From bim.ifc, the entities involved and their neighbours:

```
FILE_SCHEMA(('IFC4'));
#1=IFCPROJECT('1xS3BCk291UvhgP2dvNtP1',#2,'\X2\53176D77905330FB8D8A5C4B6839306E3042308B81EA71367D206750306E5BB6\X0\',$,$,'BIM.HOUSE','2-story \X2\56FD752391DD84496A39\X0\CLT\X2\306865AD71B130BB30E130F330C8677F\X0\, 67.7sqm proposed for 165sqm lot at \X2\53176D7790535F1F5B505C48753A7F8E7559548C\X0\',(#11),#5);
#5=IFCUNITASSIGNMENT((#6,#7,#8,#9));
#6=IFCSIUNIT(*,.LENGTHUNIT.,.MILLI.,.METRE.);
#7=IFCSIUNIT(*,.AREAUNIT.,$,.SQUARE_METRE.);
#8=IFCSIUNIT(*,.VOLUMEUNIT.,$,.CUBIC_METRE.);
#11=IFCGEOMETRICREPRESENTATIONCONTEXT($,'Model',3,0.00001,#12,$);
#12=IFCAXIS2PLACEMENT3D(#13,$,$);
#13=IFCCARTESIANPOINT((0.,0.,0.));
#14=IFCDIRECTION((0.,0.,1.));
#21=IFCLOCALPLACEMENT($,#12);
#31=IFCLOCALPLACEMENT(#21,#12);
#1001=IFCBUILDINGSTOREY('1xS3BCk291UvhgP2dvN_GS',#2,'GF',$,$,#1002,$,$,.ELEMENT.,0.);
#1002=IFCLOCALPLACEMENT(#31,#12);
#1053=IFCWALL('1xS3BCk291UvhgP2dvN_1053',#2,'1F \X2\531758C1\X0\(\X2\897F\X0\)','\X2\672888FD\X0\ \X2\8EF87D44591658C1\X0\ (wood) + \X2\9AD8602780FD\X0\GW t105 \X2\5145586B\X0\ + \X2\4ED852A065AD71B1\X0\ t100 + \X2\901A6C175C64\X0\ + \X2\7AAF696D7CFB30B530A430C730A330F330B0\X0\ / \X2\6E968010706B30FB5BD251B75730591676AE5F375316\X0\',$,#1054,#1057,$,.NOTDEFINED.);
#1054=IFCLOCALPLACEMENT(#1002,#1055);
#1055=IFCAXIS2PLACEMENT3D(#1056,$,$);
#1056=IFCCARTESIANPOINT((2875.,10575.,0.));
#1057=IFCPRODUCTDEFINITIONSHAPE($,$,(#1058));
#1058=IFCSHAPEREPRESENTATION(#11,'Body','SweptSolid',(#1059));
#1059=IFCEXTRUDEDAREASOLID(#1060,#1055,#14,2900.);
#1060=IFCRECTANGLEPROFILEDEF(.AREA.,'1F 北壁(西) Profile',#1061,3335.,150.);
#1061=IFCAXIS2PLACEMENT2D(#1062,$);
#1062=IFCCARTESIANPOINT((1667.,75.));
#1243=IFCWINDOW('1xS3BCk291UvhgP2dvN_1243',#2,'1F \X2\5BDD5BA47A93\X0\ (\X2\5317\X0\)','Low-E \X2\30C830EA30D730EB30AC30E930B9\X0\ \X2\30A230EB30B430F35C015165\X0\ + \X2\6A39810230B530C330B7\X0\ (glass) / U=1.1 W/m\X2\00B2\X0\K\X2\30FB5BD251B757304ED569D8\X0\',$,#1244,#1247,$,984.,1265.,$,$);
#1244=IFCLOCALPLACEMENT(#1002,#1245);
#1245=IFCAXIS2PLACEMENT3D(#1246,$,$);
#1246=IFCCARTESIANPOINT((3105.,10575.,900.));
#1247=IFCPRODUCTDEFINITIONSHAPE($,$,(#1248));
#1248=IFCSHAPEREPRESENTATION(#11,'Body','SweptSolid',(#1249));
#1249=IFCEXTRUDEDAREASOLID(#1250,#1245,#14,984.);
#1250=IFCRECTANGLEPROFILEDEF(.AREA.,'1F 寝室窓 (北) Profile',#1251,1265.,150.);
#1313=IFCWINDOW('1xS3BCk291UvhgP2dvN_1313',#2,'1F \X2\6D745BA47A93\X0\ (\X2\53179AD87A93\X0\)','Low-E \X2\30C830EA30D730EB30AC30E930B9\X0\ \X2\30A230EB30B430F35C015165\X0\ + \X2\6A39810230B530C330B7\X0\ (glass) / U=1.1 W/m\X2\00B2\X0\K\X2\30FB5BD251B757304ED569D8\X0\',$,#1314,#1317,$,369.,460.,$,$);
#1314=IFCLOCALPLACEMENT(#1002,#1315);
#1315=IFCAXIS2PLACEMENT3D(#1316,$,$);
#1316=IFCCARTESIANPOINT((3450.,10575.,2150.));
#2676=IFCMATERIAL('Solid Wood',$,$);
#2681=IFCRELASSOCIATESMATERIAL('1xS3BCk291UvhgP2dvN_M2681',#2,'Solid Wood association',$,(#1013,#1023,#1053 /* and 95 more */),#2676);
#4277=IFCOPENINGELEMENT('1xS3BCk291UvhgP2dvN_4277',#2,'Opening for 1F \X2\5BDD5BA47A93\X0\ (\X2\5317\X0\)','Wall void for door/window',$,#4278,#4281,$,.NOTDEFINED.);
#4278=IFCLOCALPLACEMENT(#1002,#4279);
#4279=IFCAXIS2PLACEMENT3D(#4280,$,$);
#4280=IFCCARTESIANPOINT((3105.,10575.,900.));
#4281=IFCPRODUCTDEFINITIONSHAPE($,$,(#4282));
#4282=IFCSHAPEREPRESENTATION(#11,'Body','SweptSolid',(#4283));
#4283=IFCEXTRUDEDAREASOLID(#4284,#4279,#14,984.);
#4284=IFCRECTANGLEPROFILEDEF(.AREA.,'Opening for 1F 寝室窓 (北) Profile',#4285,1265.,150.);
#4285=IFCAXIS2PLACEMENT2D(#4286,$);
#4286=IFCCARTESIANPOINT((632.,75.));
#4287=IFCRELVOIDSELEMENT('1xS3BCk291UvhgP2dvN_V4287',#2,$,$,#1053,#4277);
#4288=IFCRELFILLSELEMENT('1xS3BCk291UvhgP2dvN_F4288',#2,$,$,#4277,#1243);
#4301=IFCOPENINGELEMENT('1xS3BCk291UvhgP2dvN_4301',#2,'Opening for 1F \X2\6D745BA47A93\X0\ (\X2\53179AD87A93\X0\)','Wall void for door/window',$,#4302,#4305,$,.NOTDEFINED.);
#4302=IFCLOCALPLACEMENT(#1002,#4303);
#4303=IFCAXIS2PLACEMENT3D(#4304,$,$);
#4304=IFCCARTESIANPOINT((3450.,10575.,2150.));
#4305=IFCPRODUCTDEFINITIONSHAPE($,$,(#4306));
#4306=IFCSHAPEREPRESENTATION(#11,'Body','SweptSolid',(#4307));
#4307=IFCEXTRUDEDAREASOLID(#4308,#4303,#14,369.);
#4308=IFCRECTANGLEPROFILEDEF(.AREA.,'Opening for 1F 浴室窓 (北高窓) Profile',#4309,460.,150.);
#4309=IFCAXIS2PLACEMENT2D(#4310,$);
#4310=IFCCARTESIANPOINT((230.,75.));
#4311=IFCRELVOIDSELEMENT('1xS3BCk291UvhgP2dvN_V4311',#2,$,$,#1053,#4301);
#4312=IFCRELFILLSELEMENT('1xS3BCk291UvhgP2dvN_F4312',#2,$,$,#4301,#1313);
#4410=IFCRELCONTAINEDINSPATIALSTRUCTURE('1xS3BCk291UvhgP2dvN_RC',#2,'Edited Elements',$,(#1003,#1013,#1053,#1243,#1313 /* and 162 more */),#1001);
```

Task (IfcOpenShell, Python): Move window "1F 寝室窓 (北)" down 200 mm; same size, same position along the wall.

```python
import numpy as np
import ifcopenshell
import ifcopenshell.api.geometry
import ifcopenshell.util.placement
import ifcopenshell.util.unit

model = ifcopenshell.open("bim.ifc")
unit_scale = ifcopenshell.util.unit.calculate_unit_scale(model)

window = model.by_guid("1xS3BCk291UvhgP2dvN_1243")
opening = window.FillsVoids[0].RelatingOpeningElement
dz = -0.2 / unit_scale

shift = np.array([0.0, 0.0, dz])
# The window is not placed relative to its opening, so move both.
for product in (opening, window):
    matrix = ifcopenshell.util.placement.get_local_placement(product.ObjectPlacement)
    matrix[:3, 3] += shift
    ifcopenshell.api.geometry.edit_object_placement(model, product=product, matrix=matrix, is_si=False)

print(f"moved by {dz * unit_scale:+.3f} m")

model.write("bim_edited.ifc")
```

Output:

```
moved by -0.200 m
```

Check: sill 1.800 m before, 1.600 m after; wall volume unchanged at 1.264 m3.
